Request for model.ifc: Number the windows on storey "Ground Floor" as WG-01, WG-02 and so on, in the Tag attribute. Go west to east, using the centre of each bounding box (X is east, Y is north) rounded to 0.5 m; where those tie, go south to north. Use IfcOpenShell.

First a look at what the model holds.

```python
import ifcopenshell
import ifcopenshell.util.element
import ifcopenshell.util.placement

model = ifcopenshell.open("model.ifc")
print(model.schema)
storey = next(s for s in model.by_type("IfcBuildingStorey") if s.Name == "Ground Floor")
windows = [e for e in ifcopenshell.util.element.get_decomposition(storey) if e.is_a("IfcWindow")]
for e in sorted(windows, key=lambda e: e.id()):
    origin = ifcopenshell.util.placement.get_local_placement(e.ObjectPlacement)[:3, 3]
    print(e.id(), e.Tag, e.Name, origin.round(2) + 0.0, sep=" | ")
```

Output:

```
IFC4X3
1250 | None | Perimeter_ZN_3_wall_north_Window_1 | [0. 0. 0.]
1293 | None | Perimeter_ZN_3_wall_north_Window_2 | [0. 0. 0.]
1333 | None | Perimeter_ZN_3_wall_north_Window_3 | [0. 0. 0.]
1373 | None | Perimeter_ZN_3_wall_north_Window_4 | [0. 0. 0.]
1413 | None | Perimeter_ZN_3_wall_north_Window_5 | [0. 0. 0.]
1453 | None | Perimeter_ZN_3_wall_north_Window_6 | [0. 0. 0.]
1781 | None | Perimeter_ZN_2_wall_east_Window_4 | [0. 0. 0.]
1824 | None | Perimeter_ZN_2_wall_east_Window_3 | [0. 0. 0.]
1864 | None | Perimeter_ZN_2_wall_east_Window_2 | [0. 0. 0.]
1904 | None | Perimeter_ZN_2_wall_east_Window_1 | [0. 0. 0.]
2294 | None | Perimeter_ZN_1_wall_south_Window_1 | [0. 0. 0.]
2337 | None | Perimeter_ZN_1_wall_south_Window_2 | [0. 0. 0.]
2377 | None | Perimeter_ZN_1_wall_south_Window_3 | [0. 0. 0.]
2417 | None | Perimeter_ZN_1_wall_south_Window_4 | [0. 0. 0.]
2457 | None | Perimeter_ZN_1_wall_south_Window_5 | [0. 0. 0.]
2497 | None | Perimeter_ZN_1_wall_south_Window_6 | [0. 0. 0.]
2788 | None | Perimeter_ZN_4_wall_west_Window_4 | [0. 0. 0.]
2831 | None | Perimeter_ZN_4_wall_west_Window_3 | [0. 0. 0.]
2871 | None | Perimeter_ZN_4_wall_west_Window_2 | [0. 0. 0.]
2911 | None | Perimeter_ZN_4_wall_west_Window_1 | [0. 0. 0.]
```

```python
import ifcopenshell
import ifcopenshell.geom
import ifcopenshell.util.element
import ifcopenshell.util.shape

model = ifcopenshell.open("model.ifc")
settings = ifcopenshell.geom.settings()
settings.set("use-world-coords", True)


def centre(element):
    shape = ifcopenshell.geom.create_shape(settings, element)
    return ifcopenshell.util.shape.get_bbox_centroid(shape.geometry)


storey = next(s for s in model.by_type("IfcBuildingStorey") if s.Name == "Ground Floor")
windows = [e for e in ifcopenshell.util.element.get_decomposition(storey) if e.is_a("IfcWindow")]

# Insertion points can sit at a corner or the storey origin, so sort by the geometry (in metres).
centres = {e: centre(e) for e in windows}
windows.sort(key=lambda e: (round(centres[e][0] / 0.5), centres[e][1]))

for i, e in enumerate(windows, start=1):
    number = f"WG-{i:02d}"
    e.Tag = number
    print(e.id(), number)

model.write("model_updated.ifc")
```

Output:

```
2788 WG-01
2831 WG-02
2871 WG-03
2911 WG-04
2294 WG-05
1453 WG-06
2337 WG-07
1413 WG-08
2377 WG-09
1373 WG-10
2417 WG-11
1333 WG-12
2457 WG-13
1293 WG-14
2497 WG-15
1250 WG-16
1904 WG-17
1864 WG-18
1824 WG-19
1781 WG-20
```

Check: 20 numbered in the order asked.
